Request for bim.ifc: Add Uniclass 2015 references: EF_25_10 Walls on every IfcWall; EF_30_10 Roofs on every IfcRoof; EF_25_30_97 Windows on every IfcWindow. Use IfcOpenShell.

First a look at what the model holds.

```python
import ifcopenshell

model = ifcopenshell.open("bim.ifc")
print(model.schema)
print("classifications:", [c.Name for c in model.by_type("IfcClassification")])
for ifc_class in ("IfcDoor", "IfcRoof", "IfcStair", "IfcWall", "IfcWindow"):
    print(ifc_class, len(model.by_type(ifc_class)))
```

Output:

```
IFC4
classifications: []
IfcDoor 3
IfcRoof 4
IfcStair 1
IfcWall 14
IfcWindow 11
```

```python
import ifcopenshell
import ifcopenshell.api.classification

model = ifcopenshell.open("bim.ifc")

system = ifcopenshell.api.classification.add_classification(model, classification="Uniclass 2015")

codes = {
    "IfcWall": ("EF_25_10", "Walls"),
    "IfcRoof": ("EF_30_10", "Roofs"),
    "IfcWindow": ("EF_25_30_97", "Windows"),
}
for ifc_class, (code, name) in codes.items():
    products = model.by_type(ifc_class)
    ifcopenshell.api.classification.add_reference(
        model, products=products, classification=system, identification=code, name=name
    )
    print(code, len(products))

model.write("bim_rev.ifc")
```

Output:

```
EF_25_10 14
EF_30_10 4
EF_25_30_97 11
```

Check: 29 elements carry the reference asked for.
